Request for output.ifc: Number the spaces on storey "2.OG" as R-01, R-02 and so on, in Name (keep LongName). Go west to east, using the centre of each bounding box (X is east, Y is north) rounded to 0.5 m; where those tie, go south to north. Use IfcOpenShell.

First a look at what the model holds.

```python
import ifcopenshell
import ifcopenshell.util.element
import ifcopenshell.util.placement

model = ifcopenshell.open("output.ifc")
print(model.schema)
storey = next(s for s in model.by_type("IfcBuildingStorey") if s.Name == "2.OG")
spaces = [e for e in ifcopenshell.util.element.get_decomposition(storey) if e.is_a("IfcSpace")]
for e in sorted(spaces, key=lambda e: e.id()):
    origin = ifcopenshell.util.placement.get_local_placement(e.ObjectPlacement)[:3, 3]
    print(e.id(), e.Name, e.LongName, origin.round(2) + 0.0, sep=" | ")
```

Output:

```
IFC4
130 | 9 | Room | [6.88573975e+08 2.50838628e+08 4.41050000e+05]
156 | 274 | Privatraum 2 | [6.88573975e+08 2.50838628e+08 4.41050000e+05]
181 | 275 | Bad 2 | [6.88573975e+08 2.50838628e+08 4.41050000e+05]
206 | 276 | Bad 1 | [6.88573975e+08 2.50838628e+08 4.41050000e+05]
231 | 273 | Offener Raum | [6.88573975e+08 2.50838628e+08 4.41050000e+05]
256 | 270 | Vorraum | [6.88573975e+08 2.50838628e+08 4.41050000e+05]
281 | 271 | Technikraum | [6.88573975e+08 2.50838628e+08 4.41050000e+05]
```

```python
import ifcopenshell
import ifcopenshell.geom
import ifcopenshell.util.element
import ifcopenshell.util.shape

model = ifcopenshell.open("output.ifc")
settings = ifcopenshell.geom.settings()
settings.set("use-world-coords", True)


def centre(element):
    shape = ifcopenshell.geom.create_shape(settings, element)
    return ifcopenshell.util.shape.get_bbox_centroid(shape.geometry)


storey = next(s for s in model.by_type("IfcBuildingStorey") if s.Name == "2.OG")
spaces = [e for e in ifcopenshell.util.element.get_decomposition(storey) if e.is_a("IfcSpace")]

# Insertion points can sit at a corner or the storey origin, so sort by the geometry (in metres).
centres = {e: centre(e) for e in spaces}
spaces.sort(key=lambda e: (round(centres[e][0] / 0.5), centres[e][1]))

for i, e in enumerate(spaces, start=1):
    number = f"R-{i:02d}"
    e.Name = number
    print(e.id(), number)

model.write("output_updated.ifc")
```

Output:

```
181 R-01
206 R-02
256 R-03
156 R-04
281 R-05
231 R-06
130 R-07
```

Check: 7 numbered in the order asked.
